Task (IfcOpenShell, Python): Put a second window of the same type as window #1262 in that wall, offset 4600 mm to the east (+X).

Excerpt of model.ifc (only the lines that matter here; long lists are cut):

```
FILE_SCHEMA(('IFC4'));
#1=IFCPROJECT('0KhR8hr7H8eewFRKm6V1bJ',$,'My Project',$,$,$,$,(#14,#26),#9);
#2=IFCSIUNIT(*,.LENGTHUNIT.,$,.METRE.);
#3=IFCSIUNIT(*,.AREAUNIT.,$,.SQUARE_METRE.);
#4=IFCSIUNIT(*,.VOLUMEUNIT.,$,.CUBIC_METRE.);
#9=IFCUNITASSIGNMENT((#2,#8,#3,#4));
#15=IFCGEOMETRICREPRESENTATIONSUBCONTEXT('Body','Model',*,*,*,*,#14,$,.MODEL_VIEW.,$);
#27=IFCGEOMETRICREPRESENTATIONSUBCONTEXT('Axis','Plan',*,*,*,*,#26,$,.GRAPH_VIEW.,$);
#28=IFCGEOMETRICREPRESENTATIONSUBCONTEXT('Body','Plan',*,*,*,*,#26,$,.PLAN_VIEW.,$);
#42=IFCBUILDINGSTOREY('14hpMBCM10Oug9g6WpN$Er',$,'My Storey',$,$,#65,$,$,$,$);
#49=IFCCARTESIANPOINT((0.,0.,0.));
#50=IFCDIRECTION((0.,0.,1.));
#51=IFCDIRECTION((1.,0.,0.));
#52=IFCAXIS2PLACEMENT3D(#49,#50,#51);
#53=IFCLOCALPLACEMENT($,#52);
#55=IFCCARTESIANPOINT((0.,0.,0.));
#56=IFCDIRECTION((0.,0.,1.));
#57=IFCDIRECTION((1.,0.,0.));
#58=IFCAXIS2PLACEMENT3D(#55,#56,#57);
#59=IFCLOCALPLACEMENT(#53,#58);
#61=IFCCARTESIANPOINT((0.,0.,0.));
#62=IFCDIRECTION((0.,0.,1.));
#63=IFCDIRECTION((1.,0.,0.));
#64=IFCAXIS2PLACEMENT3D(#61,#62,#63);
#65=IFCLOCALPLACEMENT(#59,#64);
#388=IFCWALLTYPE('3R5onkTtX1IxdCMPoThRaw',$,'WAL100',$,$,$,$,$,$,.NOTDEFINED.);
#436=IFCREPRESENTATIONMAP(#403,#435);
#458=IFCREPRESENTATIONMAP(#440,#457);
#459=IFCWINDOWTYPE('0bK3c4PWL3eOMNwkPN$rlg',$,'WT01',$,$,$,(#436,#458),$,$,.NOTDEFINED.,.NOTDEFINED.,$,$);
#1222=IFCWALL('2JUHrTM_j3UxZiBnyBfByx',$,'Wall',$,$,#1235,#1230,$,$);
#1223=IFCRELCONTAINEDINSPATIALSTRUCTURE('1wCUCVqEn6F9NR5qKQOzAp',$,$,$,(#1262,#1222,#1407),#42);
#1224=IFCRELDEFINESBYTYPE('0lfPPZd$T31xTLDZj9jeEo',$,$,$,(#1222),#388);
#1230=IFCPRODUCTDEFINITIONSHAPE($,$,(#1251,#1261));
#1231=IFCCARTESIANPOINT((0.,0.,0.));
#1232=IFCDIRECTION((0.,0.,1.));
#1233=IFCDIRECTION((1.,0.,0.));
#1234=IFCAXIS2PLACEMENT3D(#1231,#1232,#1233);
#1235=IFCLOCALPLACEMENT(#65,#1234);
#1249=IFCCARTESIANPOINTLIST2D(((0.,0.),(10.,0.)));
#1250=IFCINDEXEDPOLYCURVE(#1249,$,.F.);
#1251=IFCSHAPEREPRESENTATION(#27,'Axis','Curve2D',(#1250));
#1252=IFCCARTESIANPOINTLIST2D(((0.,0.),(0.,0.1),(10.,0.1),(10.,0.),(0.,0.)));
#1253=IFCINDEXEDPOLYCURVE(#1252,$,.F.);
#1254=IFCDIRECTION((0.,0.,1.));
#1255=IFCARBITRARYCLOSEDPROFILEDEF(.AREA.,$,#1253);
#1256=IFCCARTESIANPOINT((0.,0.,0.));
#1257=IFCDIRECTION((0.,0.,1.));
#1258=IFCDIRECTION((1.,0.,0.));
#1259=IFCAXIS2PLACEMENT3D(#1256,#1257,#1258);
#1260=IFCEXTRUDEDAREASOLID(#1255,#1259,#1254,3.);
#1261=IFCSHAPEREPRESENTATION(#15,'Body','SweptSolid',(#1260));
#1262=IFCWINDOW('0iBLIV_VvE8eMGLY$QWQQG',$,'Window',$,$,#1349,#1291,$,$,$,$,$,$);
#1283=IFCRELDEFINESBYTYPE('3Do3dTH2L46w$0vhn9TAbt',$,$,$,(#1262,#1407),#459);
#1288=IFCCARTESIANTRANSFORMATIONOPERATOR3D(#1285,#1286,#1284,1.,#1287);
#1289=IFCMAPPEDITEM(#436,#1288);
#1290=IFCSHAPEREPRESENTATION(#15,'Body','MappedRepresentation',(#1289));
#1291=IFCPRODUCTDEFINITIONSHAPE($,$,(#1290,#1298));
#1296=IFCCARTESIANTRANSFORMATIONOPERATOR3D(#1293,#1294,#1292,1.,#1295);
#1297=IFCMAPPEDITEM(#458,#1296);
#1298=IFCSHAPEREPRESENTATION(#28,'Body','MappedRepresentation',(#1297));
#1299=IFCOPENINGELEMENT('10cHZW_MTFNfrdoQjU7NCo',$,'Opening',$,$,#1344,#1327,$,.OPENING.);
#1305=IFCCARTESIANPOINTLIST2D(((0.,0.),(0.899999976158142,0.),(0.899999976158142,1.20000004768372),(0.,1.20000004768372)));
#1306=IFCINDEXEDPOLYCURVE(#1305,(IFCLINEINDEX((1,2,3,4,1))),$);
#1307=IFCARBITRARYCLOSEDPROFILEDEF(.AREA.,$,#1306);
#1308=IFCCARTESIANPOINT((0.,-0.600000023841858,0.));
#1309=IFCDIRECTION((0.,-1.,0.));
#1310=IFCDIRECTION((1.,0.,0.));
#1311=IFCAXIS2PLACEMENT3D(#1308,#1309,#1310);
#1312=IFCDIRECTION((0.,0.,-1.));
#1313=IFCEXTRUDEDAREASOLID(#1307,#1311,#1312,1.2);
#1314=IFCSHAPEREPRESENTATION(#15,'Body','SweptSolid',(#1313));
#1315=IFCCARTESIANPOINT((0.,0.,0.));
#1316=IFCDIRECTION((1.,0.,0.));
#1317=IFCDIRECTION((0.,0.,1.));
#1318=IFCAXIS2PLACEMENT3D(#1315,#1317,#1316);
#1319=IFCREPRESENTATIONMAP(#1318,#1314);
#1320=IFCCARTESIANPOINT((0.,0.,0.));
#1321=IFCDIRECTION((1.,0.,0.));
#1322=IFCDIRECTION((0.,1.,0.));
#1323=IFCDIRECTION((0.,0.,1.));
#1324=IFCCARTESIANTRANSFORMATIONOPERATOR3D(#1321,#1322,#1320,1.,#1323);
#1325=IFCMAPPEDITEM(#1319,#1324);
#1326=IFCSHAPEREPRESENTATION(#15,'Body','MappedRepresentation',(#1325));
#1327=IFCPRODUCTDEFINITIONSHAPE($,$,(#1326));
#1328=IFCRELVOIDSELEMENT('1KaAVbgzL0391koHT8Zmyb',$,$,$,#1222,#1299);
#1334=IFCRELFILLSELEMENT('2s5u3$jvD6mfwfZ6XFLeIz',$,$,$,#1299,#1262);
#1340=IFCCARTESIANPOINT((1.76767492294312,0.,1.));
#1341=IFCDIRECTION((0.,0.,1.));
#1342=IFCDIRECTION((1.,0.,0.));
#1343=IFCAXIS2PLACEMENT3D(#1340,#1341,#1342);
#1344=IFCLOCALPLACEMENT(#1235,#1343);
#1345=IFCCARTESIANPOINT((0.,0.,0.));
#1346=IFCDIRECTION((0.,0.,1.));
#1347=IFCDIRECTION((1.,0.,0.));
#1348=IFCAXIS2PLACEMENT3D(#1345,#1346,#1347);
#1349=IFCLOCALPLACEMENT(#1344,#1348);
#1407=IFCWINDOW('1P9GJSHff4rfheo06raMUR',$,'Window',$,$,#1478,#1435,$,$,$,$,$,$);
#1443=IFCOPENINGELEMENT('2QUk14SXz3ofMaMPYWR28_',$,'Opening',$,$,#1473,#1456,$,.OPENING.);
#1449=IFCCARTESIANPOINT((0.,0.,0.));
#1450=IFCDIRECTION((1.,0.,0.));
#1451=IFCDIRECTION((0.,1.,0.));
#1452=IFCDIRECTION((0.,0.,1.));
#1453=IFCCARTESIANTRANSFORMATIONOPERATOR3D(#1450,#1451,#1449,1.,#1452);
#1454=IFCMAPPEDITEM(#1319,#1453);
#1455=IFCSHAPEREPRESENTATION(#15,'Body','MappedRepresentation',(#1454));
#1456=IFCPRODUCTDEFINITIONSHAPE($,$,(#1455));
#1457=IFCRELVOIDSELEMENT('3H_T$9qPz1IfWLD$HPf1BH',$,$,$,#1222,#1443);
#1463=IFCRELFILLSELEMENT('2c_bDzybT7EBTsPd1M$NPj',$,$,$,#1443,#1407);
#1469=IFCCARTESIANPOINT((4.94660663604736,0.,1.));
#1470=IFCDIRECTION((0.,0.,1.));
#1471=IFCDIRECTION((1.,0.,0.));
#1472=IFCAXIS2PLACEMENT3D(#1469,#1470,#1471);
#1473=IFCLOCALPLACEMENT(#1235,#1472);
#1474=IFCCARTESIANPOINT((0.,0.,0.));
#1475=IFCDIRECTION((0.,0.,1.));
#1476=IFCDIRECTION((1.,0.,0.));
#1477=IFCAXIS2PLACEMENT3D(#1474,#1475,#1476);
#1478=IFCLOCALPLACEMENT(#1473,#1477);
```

```python
import ifcopenshell
import ifcopenshell.api.feature
import ifcopenshell.api.geometry
import ifcopenshell.api.root
import ifcopenshell.geom
import ifcopenshell.util.element
import ifcopenshell.util.placement
import ifcopenshell.util.shape
import ifcopenshell.util.unit

model = ifcopenshell.open("model.ifc")
unit_scale = ifcopenshell.util.unit.calculate_unit_scale(model)
settings = ifcopenshell.geom.settings()


def volume(element):
    """Net volume in cubic metres, openings subtracted."""
    shape = ifcopenshell.geom.create_shape(settings, element)
    return ifcopenshell.util.shape.get_volume(shape.geometry)


window = model.by_id(1262)
opening = window.FillsVoids[0].RelatingOpeningElement
wall = opening.VoidsElements[0].RelatingBuildingElement
before = volume(wall)
shift = ifcopenshell.util.placement.get_local_placement(wall.ObjectPlacement)[:3, 0] * 4.6 / unit_scale

# copy_class copies the void relationship, type, container and properties, but no geometry.
new_opening = ifcopenshell.api.root.copy_class(model, product=opening)
new_opening.Representation = ifcopenshell.util.element.copy_deep(
    model, opening.Representation, exclude=["IfcGeometricRepresentationContext", "IfcRepresentationMap"]
)
new_window = ifcopenshell.api.root.copy_class(model, product=window)
new_window.Representation = ifcopenshell.util.element.copy_deep(
    model, window.Representation, exclude=["IfcGeometricRepresentationContext", "IfcRepresentationMap"]
)
ifcopenshell.api.feature.add_filling(model, opening=new_opening, element=new_window)

for old, new in ((opening, new_opening), (window, new_window)):
    matrix = ifcopenshell.util.placement.get_local_placement(old.ObjectPlacement)
    matrix[:3, 3] += shift
    ifcopenshell.api.geometry.edit_object_placement(model, product=new, matrix=matrix, is_si=False)

after = volume(wall)

print(f"wall volume {before:.3f} -> {after:.3f} m3")

model.write("model_updated.ifc")
```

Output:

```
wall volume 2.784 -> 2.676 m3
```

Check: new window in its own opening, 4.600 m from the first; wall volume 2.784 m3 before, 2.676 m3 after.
